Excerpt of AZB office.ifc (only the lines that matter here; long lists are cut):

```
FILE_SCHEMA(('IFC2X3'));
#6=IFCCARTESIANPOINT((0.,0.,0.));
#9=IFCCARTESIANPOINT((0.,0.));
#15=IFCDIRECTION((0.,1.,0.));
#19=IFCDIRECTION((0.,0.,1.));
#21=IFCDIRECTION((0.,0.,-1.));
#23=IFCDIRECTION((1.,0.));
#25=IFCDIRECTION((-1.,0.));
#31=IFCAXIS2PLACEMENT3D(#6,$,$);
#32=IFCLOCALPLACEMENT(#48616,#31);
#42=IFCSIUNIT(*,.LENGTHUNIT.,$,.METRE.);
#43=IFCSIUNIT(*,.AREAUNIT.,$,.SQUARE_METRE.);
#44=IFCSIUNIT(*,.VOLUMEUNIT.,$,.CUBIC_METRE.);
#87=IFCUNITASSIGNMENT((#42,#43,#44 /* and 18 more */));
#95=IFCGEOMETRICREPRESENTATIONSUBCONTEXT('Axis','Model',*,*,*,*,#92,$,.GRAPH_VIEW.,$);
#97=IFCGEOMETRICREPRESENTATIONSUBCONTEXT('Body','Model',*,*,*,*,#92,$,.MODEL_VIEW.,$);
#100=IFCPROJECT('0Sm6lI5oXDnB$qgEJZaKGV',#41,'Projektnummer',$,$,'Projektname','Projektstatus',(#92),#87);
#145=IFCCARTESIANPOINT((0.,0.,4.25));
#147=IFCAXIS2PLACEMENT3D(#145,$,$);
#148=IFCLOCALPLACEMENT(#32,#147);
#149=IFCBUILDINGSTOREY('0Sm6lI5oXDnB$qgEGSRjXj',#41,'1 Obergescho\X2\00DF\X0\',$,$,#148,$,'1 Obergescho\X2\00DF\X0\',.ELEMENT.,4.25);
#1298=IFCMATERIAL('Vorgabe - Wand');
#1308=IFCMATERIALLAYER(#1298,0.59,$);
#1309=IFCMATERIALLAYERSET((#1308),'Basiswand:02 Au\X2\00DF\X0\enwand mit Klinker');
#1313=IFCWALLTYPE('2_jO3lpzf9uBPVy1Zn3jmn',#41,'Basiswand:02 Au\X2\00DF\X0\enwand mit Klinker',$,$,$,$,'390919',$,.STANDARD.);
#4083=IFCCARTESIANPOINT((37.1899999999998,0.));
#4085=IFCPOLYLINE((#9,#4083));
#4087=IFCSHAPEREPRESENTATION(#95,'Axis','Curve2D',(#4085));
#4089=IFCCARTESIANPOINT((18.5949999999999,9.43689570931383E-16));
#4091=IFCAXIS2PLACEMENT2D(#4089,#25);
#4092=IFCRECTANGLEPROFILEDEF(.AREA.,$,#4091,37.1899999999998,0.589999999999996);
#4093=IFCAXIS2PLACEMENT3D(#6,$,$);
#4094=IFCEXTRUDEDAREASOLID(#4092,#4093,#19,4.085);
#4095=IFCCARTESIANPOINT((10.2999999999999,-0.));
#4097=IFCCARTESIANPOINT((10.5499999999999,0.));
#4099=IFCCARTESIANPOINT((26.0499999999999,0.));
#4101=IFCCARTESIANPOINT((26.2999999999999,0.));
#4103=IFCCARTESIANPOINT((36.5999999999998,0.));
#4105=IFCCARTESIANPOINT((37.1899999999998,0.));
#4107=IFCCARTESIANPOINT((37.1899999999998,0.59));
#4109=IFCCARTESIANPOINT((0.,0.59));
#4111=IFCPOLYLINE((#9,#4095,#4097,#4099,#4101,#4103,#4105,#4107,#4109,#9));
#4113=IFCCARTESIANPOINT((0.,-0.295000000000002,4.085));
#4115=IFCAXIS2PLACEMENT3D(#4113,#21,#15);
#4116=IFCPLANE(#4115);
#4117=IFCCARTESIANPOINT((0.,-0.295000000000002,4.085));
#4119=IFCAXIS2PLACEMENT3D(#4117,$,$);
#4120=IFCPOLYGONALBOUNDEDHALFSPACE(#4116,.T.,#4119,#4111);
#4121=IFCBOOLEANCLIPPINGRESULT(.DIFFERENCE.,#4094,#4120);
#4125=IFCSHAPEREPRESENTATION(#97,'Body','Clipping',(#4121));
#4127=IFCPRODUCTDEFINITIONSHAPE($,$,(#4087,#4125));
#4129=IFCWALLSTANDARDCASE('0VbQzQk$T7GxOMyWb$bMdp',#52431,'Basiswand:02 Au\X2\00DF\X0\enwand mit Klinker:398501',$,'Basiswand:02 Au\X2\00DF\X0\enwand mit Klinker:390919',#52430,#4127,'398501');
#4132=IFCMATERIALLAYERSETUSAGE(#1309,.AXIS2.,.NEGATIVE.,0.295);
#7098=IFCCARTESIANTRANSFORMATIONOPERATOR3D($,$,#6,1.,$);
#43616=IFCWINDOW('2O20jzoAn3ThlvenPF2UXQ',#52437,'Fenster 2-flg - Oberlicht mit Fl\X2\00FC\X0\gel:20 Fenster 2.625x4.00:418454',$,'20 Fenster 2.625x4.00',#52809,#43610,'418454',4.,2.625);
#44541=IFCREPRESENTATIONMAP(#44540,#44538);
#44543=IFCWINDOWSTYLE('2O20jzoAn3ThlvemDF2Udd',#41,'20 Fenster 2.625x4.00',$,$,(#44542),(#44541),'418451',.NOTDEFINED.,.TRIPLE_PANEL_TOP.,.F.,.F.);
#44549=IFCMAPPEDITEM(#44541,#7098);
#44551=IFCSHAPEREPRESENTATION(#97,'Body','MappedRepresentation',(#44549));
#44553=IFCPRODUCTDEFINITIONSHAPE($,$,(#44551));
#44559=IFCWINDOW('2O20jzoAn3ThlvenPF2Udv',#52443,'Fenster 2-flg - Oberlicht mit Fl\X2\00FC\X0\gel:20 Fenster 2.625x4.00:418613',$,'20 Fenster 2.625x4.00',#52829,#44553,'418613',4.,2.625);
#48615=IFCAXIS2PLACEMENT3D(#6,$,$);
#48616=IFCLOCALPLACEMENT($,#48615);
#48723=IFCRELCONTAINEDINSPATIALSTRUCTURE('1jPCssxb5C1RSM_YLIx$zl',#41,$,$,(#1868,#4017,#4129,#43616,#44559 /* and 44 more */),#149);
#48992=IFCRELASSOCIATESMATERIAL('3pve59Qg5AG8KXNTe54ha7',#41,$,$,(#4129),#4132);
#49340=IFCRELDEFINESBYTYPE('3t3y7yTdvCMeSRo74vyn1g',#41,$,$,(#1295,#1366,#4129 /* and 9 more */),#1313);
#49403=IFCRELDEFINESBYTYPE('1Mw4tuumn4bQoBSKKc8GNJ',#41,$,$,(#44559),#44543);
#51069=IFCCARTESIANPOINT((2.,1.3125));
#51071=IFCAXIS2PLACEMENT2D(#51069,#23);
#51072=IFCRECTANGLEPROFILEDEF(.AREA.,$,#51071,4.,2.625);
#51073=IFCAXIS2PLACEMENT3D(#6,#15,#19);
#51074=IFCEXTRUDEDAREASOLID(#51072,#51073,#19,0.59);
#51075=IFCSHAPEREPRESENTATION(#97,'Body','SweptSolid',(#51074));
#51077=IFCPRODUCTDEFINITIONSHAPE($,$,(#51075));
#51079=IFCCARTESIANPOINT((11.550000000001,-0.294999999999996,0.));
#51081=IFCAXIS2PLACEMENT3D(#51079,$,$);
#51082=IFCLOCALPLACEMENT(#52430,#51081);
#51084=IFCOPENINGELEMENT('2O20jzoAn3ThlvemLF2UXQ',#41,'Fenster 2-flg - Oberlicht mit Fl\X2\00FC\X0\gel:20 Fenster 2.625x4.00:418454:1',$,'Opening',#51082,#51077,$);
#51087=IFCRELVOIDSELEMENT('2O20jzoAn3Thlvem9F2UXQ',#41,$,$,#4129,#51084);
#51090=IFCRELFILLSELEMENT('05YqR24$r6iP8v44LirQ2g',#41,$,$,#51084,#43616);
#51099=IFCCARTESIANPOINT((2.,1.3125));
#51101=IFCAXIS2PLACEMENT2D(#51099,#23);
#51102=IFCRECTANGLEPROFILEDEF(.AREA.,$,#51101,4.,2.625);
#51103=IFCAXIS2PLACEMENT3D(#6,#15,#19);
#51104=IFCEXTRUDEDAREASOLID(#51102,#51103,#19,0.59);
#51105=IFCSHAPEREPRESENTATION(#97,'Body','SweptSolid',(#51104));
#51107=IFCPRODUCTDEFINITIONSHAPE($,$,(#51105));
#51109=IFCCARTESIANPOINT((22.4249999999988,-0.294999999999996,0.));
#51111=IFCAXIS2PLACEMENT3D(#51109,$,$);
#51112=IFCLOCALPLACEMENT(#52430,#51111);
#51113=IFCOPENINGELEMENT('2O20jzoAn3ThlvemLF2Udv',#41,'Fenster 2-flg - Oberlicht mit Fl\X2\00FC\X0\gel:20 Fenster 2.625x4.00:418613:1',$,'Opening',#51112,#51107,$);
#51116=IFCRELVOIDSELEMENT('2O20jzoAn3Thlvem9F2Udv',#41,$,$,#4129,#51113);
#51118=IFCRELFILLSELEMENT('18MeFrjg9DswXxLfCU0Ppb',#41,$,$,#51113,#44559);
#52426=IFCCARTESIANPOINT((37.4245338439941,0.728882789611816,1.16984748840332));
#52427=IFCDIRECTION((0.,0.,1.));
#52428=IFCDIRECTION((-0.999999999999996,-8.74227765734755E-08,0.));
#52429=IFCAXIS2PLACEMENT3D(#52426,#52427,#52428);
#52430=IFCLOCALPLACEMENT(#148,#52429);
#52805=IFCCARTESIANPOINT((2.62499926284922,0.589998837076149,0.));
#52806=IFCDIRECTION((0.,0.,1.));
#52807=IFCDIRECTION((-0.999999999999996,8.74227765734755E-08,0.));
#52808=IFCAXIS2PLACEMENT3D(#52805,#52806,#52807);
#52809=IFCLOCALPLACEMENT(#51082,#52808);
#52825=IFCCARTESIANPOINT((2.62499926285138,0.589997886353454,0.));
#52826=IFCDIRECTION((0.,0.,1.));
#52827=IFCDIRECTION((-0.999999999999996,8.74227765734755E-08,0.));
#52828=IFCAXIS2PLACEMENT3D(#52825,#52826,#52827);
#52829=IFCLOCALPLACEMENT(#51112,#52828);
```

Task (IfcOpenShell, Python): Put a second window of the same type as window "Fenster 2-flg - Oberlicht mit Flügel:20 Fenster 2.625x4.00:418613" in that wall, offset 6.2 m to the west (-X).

```python
import ifcopenshell
import ifcopenshell.api.feature
import ifcopenshell.api.geometry
import ifcopenshell.api.root
import ifcopenshell.geom
import ifcopenshell.util.element
import ifcopenshell.util.placement
import ifcopenshell.util.shape

model = ifcopenshell.open("AZB office.ifc")
settings = ifcopenshell.geom.settings()


def volume(element):
    """Net volume in cubic metres, openings subtracted."""
    shape = ifcopenshell.geom.create_shape(settings, element)
    return ifcopenshell.util.shape.get_volume(shape.geometry)


def reuse_history(source, copy):
    """copy_class also copies each property set's owner history, people and application; keep the originals."""
    for rel in copy.IsDefinedBy:
        if rel.is_a("IfcRelDefinesByProperties") and (history := rel.RelatingPropertyDefinition.OwnerHistory):
            rel.RelatingPropertyDefinition.OwnerHistory = source.OwnerHistory
            ifcopenshell.util.element.remove_deep2(model, history)


window = model.by_guid("2O20jzoAn3ThlvenPF2Udv")
opening = window.FillsVoids[0].RelatingOpeningElement
wall = opening.VoidsElements[0].RelatingBuildingElement
before = volume(wall)
shift = ifcopenshell.util.placement.get_local_placement(wall.ObjectPlacement)[:3, 0] * 6.2

# copy_class copies the void relationship, type, container and properties, but no geometry.
new_opening = ifcopenshell.api.root.copy_class(model, product=opening)
new_opening.Representation = ifcopenshell.util.element.copy_deep(
    model, opening.Representation, exclude=["IfcGeometricRepresentationContext", "IfcRepresentationMap"]
)
new_opening.Name = "Fenster 2-flg - Oberlicht mit Flügel:20 Fenster 2.625x4.00"
new_window = ifcopenshell.api.root.copy_class(model, product=window)
new_window.Representation = ifcopenshell.util.element.copy_deep(
    model, window.Representation, exclude=["IfcGeometricRepresentationContext", "IfcRepresentationMap"]
)
new_window.Name = "Fenster 2-flg - Oberlicht mit Flügel:20 Fenster 2.625x4.00"
new_window.Tag = None
reuse_history(window, new_window)
fills = ifcopenshell.api.feature.add_filling(model, opening=new_opening, element=new_window)
fills.OwnerHistory = new_window.OwnerHistory  # required in IFC2X3

for old, new in ((opening, new_opening), (window, new_window)):
    matrix = ifcopenshell.util.placement.get_local_placement(old.ObjectPlacement)
    matrix[:3, 3] += shift
    ifcopenshell.api.geometry.edit_object_placement(model, product=new, matrix=matrix, is_si=False)

after = volume(wall)

print(f"wall volume {before:.3f} -> {after:.3f} m3")

model.write("AZB office_edited.ifc")
```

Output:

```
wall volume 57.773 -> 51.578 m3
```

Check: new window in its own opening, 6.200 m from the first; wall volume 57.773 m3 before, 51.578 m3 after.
